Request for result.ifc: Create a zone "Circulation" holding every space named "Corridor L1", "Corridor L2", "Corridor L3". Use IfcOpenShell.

First a look at what the model holds.

```python
import ifcopenshell

model = ifcopenshell.open("result.ifc")
print(model.schema)
seen = {}
for space in model.by_type("IfcSpace"):
    seen[space.Name] = seen.get(space.Name, 0) + 1
for name, count in sorted(seen.items(), key=str):
    print(count, "x", name)
print("zones:", [z.Name for z in model.by_type("IfcZone")][:20])
```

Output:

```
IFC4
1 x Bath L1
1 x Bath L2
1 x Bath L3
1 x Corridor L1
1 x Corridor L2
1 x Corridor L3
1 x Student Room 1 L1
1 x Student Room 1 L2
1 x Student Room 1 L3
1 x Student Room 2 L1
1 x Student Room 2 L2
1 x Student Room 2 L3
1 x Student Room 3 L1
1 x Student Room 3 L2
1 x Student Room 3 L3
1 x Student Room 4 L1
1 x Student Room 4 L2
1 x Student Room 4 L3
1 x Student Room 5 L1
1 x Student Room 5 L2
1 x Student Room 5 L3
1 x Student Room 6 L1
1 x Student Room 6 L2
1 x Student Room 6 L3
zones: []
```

```python
import ifcopenshell
import ifcopenshell.api.group
import ifcopenshell.api.root

model = ifcopenshell.open("result.ifc")

names = {"Corridor L1", "Corridor L2", "Corridor L3"}
spaces = [s for s in model.by_type("IfcSpace") if s.Name in names]

zone = ifcopenshell.api.root.create_entity(model, ifc_class="IfcZone", name="Circulation")
ifcopenshell.api.group.assign_group(model, products=spaces, group=zone)
print(len(spaces), "spaces in", zone.Name)

model.write("result_v2.ifc")
```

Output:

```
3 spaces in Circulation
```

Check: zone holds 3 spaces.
